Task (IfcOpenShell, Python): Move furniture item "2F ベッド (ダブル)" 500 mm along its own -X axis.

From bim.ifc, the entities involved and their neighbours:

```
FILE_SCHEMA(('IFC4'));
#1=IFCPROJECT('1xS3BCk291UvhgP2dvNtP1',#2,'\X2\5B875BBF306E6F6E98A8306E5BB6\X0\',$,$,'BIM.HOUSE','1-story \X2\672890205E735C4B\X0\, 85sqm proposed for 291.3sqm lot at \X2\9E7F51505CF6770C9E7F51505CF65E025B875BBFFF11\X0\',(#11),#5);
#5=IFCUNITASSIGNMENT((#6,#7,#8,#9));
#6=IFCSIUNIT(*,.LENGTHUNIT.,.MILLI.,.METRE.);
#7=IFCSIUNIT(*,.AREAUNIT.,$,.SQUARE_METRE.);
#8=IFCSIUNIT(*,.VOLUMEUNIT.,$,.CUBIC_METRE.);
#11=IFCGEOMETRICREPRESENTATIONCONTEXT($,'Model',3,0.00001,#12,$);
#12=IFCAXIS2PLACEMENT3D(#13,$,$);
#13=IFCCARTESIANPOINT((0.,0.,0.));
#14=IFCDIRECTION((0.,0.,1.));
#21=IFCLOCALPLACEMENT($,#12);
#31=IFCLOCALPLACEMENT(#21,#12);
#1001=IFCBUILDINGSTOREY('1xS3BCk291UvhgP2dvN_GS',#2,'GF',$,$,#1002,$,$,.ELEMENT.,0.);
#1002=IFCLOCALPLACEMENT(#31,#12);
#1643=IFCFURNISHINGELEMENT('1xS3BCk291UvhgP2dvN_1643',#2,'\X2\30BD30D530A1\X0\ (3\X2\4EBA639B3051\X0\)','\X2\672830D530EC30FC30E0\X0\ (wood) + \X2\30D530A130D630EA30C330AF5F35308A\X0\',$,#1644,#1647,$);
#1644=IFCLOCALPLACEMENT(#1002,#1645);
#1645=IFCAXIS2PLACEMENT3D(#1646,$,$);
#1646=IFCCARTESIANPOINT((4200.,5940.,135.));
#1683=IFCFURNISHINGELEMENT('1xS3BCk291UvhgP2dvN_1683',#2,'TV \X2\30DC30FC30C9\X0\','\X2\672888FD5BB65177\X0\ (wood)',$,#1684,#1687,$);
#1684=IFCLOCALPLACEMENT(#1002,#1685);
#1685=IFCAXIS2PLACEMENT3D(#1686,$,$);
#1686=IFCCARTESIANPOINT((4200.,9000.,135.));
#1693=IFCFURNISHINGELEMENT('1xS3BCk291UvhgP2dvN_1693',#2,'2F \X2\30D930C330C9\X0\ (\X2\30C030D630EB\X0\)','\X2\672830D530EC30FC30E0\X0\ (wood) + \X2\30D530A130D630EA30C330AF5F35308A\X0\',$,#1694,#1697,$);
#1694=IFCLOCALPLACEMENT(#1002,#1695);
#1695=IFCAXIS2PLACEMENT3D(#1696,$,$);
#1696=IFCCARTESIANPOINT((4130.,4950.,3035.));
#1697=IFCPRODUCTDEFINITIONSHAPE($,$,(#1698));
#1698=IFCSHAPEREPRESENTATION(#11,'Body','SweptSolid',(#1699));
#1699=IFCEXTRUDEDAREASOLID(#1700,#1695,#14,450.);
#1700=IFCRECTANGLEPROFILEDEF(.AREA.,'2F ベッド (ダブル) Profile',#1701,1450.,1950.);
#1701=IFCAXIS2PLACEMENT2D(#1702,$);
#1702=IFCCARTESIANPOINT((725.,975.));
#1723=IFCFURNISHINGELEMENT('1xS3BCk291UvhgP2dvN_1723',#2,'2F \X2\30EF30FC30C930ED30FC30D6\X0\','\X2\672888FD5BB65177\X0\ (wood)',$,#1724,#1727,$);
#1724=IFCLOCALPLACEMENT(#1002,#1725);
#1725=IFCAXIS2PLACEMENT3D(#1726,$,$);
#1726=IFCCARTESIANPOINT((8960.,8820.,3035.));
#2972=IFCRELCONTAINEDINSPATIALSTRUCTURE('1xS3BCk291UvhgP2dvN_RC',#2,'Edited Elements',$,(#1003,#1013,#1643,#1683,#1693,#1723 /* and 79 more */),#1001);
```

```python
import ifcopenshell
import ifcopenshell.api.geometry
import ifcopenshell.util.placement

model = ifcopenshell.open("bim.ifc")

item = model.by_guid("1xS3BCk291UvhgP2dvN_1693")
matrix = ifcopenshell.util.placement.get_local_placement(item.ObjectPlacement)
matrix[:3, 3] -= matrix[:3, 0] * 500.0
ifcopenshell.api.geometry.edit_object_placement(model, product=item, matrix=matrix, is_si=False)

print(ifcopenshell.util.placement.get_local_placement(item.ObjectPlacement).round(3) + 0.0)

model.write("bim_updated.ifc")
```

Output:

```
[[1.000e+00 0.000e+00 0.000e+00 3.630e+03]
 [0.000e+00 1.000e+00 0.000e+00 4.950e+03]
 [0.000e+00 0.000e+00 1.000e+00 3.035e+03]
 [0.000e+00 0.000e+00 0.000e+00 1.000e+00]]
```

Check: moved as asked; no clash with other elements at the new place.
